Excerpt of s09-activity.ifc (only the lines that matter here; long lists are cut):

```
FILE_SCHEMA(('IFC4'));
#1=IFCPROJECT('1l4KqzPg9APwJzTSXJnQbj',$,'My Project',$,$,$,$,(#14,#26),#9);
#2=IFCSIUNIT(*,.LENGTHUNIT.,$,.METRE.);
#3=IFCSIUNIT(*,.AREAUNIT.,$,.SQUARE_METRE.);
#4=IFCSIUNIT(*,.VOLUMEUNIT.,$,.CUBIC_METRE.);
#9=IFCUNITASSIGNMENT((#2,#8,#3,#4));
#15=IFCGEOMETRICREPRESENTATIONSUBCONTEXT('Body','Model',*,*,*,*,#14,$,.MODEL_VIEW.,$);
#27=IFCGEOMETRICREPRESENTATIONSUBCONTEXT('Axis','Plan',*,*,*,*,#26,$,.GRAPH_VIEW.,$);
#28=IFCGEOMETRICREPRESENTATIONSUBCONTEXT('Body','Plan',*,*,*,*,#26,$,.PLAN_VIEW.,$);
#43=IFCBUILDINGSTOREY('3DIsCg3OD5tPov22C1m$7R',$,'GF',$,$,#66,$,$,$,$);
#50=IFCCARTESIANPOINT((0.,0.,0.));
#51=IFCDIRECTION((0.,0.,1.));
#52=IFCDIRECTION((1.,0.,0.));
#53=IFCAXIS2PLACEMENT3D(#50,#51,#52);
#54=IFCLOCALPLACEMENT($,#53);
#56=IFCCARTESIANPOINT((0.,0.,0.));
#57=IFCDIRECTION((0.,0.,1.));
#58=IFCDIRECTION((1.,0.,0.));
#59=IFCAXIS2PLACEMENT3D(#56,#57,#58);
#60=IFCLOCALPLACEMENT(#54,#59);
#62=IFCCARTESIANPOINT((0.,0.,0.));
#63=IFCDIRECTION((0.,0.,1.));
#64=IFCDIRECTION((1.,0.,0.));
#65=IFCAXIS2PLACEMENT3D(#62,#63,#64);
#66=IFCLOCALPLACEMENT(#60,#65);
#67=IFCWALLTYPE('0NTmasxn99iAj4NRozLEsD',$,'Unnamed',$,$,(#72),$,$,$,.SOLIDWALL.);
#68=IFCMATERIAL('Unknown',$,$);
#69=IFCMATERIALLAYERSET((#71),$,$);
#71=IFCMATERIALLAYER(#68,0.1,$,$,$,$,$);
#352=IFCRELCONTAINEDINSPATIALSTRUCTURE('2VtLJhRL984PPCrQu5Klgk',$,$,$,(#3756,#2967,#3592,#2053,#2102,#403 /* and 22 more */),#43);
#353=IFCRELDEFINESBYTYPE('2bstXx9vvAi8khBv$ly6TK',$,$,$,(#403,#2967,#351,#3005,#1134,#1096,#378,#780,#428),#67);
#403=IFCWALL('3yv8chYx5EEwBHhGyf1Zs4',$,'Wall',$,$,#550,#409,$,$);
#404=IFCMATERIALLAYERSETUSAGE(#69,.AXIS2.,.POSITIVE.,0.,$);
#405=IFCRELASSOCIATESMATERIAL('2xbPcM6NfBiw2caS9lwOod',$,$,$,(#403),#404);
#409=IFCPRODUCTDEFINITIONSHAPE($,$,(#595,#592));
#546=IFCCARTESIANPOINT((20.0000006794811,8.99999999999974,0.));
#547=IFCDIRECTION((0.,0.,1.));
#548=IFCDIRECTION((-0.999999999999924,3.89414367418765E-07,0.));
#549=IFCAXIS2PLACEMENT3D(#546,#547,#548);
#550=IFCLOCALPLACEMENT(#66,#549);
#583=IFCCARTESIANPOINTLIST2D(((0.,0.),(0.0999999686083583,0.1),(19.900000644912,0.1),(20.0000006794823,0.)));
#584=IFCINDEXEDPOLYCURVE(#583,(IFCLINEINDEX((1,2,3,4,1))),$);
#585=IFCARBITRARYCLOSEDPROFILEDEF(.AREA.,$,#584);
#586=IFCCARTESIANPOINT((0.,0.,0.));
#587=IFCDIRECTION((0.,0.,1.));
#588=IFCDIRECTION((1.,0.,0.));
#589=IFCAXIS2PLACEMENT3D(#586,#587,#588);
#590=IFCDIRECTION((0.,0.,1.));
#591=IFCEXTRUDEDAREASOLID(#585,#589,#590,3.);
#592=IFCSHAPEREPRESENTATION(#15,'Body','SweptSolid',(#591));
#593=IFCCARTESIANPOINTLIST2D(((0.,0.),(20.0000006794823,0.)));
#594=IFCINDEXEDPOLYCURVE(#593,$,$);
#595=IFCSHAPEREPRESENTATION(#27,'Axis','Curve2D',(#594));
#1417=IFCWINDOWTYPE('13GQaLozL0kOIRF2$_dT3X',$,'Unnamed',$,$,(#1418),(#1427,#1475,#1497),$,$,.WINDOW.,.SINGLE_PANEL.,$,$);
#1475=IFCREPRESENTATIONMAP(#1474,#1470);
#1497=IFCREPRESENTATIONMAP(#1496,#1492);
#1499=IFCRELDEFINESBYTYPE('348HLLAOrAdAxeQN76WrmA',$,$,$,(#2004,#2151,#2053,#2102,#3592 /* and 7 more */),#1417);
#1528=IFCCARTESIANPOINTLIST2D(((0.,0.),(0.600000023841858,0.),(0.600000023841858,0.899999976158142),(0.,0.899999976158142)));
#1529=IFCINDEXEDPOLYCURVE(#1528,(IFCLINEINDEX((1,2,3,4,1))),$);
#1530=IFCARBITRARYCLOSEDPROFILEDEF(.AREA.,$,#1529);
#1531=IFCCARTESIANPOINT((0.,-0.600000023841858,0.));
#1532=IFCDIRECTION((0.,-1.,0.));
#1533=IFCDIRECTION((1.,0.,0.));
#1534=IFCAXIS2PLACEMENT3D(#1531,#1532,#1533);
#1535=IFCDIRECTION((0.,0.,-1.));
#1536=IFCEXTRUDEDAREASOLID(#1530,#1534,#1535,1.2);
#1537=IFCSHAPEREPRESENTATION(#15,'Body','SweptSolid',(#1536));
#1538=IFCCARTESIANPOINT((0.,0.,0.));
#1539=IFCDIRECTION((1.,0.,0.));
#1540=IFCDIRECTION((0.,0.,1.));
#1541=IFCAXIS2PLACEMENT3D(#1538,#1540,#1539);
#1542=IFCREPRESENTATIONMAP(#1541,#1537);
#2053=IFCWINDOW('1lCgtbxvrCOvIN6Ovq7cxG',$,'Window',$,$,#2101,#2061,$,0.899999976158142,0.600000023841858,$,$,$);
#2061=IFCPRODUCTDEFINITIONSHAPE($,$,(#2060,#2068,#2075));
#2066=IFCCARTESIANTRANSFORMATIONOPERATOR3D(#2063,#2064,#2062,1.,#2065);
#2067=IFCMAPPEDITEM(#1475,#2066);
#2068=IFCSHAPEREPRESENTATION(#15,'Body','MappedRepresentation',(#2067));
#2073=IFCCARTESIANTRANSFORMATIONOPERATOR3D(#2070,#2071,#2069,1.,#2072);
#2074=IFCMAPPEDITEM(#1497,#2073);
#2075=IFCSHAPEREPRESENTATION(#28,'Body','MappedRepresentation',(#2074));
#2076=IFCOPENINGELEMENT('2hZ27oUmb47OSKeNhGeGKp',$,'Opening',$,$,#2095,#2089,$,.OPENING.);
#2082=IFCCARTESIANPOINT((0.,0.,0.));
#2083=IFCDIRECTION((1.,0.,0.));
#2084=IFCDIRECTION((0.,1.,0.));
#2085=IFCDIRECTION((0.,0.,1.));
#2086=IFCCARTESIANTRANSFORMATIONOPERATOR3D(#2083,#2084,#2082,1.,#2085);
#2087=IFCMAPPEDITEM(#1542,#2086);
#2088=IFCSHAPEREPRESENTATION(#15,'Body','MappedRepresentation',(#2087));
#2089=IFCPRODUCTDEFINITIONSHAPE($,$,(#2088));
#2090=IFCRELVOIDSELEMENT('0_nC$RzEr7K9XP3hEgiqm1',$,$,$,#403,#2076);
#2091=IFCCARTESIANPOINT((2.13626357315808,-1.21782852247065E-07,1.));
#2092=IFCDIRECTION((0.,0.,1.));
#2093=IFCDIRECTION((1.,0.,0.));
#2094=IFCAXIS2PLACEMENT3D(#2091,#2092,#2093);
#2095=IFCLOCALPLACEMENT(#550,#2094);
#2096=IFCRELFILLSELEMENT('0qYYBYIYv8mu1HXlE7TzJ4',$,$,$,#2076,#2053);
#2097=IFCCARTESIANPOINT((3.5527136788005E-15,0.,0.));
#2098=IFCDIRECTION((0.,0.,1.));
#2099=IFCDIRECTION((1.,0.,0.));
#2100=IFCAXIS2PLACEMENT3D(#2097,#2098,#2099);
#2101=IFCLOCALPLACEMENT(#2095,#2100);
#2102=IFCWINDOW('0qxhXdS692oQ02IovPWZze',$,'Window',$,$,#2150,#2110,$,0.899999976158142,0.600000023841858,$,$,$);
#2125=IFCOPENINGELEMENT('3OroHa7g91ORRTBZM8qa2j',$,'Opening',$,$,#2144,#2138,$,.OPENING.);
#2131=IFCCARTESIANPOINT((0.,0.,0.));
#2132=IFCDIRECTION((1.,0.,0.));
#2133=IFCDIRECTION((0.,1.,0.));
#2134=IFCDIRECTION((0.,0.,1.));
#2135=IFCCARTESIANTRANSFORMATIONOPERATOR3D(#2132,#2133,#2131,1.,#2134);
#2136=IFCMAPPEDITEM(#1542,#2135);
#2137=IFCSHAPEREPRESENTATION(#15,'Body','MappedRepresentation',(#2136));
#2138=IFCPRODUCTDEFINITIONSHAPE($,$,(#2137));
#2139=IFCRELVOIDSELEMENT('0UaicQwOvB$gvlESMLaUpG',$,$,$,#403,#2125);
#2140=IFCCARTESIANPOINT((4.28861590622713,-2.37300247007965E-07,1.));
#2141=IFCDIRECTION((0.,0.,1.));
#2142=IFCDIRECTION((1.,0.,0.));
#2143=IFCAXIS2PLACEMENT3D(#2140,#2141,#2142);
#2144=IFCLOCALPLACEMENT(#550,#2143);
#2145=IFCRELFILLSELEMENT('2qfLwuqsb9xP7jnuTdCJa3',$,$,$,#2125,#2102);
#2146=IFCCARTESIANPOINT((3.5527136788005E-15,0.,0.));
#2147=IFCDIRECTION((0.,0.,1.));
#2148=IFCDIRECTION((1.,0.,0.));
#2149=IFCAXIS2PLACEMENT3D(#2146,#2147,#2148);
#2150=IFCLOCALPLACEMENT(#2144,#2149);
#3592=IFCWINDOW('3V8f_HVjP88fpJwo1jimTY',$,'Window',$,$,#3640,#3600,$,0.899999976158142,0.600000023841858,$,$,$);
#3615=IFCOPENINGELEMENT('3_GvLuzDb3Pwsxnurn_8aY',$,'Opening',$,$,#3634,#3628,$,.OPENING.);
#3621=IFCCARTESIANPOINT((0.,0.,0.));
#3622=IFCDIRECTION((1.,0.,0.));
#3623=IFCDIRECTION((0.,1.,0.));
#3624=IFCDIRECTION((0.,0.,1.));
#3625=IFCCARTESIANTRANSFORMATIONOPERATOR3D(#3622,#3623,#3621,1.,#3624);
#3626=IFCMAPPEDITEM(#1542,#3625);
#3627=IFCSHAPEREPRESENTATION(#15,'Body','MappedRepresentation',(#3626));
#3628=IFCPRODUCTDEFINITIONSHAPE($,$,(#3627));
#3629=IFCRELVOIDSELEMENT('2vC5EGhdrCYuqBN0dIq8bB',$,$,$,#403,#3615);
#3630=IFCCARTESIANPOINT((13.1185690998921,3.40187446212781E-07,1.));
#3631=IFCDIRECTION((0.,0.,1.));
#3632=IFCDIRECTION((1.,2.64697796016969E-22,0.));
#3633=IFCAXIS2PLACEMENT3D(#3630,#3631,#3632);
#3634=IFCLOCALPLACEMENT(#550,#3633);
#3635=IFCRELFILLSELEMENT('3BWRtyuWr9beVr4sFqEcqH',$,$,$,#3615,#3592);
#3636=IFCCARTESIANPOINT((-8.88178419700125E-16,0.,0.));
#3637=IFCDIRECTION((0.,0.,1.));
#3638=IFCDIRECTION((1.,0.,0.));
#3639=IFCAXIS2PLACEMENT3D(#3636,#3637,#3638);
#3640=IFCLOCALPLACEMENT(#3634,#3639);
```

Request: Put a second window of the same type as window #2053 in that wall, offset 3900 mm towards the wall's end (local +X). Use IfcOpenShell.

```python
import ifcopenshell
import ifcopenshell.api.feature
import ifcopenshell.api.geometry
import ifcopenshell.api.root
import ifcopenshell.geom
import ifcopenshell.util.element
import ifcopenshell.util.placement
import ifcopenshell.util.shape
import ifcopenshell.util.unit

model = ifcopenshell.open("s09-activity.ifc")
unit_scale = ifcopenshell.util.unit.calculate_unit_scale(model)
settings = ifcopenshell.geom.settings()


def volume(element):
    """Net volume in cubic metres, openings subtracted."""
    shape = ifcopenshell.geom.create_shape(settings, element)
    return ifcopenshell.util.shape.get_volume(shape.geometry)


window = model.by_guid("1lCgtbxvrCOvIN6Ovq7cxG")
opening = window.FillsVoids[0].RelatingOpeningElement
wall = opening.VoidsElements[0].RelatingBuildingElement
before = volume(wall)
shift = ifcopenshell.util.placement.get_local_placement(wall.ObjectPlacement)[:3, 0] * 3.9 / unit_scale

# copy_class copies the void relationship, type, container and properties, but no geometry.
new_opening = ifcopenshell.api.root.copy_class(model, product=opening)
new_opening.Representation = ifcopenshell.util.element.copy_deep(
    model, opening.Representation, exclude=["IfcGeometricRepresentationContext", "IfcRepresentationMap"]
)
new_window = ifcopenshell.api.root.copy_class(model, product=window)
new_window.Representation = ifcopenshell.util.element.copy_deep(
    model, window.Representation, exclude=["IfcGeometricRepresentationContext", "IfcRepresentationMap"]
)
ifcopenshell.api.feature.add_filling(model, opening=new_opening, element=new_window)

for old, new in ((opening, new_opening), (window, new_window)):
    matrix = ifcopenshell.util.placement.get_local_placement(old.ObjectPlacement)
    matrix[:3, 3] += shift
    ifcopenshell.api.geometry.edit_object_placement(model, product=new, matrix=matrix, is_si=False)

after = volume(wall)

print(f"wall volume {before:.3f} -> {after:.3f} m3")

model.write("s09-activity_updated.ifc")
```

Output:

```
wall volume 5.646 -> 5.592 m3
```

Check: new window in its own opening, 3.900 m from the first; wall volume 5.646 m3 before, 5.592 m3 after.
